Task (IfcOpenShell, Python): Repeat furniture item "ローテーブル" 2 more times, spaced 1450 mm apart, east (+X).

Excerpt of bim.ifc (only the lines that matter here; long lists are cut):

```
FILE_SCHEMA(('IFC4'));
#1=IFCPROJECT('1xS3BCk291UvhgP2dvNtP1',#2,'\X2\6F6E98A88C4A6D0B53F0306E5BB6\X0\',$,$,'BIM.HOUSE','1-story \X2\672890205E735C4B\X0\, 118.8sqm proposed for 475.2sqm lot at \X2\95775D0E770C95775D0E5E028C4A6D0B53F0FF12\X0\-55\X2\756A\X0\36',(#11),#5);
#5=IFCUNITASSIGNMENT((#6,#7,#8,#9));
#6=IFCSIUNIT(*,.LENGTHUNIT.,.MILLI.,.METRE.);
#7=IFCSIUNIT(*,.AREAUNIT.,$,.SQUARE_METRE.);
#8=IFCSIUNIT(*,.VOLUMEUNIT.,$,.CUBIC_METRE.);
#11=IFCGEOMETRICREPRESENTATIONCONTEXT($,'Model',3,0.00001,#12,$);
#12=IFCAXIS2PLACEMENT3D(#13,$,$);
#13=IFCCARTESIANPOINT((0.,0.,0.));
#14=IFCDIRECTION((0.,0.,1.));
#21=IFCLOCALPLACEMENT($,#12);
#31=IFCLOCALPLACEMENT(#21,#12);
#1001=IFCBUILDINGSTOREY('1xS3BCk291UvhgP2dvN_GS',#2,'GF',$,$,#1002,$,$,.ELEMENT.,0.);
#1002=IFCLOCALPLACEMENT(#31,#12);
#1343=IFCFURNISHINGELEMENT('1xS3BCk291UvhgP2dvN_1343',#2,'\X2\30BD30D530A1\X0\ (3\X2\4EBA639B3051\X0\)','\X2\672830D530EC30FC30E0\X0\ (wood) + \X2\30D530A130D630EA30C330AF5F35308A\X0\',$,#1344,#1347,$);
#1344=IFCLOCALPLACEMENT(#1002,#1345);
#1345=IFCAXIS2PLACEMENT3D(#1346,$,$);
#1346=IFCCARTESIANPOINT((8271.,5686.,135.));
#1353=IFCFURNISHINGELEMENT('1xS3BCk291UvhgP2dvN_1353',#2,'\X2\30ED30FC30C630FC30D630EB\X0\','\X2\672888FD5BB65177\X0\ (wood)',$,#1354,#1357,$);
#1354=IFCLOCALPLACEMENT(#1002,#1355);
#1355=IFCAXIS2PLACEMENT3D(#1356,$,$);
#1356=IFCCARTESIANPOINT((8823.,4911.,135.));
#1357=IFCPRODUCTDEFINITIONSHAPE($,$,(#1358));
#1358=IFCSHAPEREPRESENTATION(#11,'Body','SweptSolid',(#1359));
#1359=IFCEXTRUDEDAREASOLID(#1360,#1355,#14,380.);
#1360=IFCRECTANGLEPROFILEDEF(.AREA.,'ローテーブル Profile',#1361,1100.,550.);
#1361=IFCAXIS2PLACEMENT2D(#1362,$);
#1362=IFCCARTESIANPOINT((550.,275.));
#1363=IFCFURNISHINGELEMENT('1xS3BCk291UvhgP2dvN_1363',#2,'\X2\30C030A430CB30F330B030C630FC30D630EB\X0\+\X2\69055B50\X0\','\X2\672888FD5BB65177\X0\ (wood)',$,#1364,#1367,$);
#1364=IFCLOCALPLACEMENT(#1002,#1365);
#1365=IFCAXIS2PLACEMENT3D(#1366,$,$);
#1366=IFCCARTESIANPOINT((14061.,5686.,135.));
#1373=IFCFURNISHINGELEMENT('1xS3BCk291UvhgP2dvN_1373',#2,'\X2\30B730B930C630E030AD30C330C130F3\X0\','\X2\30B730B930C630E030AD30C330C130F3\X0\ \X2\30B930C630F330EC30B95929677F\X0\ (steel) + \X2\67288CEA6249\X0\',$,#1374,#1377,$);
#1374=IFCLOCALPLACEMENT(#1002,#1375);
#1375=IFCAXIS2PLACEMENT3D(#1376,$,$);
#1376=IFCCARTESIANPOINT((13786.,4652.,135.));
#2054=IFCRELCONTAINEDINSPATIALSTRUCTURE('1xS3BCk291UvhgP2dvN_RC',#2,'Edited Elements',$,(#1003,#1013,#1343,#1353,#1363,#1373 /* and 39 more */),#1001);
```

```python
import numpy as np
import ifcopenshell
import ifcopenshell.api.geometry
import ifcopenshell.api.root
import ifcopenshell.util.element
import ifcopenshell.util.placement

model = ifcopenshell.open("bim.ifc")


def reuse_history(source, copy):
    """copy_class also copies each property set's owner history, people and application; keep the originals."""
    for rel in copy.IsDefinedBy:
        if rel.is_a("IfcRelDefinesByProperties") and (history := rel.RelatingPropertyDefinition.OwnerHistory):
            rel.RelatingPropertyDefinition.OwnerHistory = source.OwnerHistory
            ifcopenshell.util.element.remove_deep2(model, history)


source = model.by_guid("1xS3BCk291UvhgP2dvN_1353")
base = ifcopenshell.util.placement.get_local_placement(source.ObjectPlacement)
step = np.array([1.0, 0.0, 0.0]) * 1450.0

for i in range(1, 3):
    copy = ifcopenshell.api.root.copy_class(model, product=source)
    copy.Representation = ifcopenshell.util.element.copy_deep(
        model, source.Representation, exclude=["IfcGeometricRepresentationContext", "IfcRepresentationMap"]
    )
    reuse_history(source, copy)
    matrix = base.copy()
    matrix[:3, 3] += i * step
    print("added at", matrix[:3, 3].round(3) + 0.0)
    ifcopenshell.api.geometry.edit_object_placement(model, product=copy, matrix=matrix, is_si=False)

model.write("bim_v2.ifc")
```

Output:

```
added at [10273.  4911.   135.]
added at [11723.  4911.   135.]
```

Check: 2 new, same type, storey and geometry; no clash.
